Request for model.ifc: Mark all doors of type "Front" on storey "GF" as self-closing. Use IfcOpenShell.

First a look at what the model holds.

```python
import ifcopenshell
import ifcopenshell.util.element

model = ifcopenshell.open("model.ifc")
print(model.schema)
storey = next(s for s in model.by_type("IfcBuildingStorey") if s.Name == "GF")
doors = [e for e in ifcopenshell.util.element.get_decomposition(storey) if e.is_a("IfcDoor")]
seen = {}
for e in doors:
    element_type = ifcopenshell.util.element.get_type(e)
    key = (element_type.Name if element_type != e and element_type else None, ifcopenshell.util.element.get_pset(e, "Pset_DoorCommon", "SelfClosing"))
    seen[key] = seen.get(key, 0) + 1
for (name, value), count in sorted(seen.items(), key=str):
    print(count, "x", name, "|", value)
```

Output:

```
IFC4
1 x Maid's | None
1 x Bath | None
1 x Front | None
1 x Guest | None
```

```python
import ifcopenshell
import ifcopenshell.api.pset
import ifcopenshell.util.element

model = ifcopenshell.open("model.ifc")

storey = next(s for s in model.by_type("IfcBuildingStorey") if s.Name == "GF")
doors = [e for e in ifcopenshell.util.element.get_decomposition(storey) if e.is_a("IfcDoor")]

count = 0
for e in doors:
    element_type = ifcopenshell.util.element.get_type(e)
    if element_type in (None, e) or element_type.Name != "Front":
        continue
    # add_pset returns the element's existing set when there is one.
    pset = ifcopenshell.api.pset.add_pset(model, product=e, name="Pset_DoorCommon")
    ifcopenshell.api.pset.edit_pset(model, pset=pset, properties={"SelfClosing": True})
    count += 1

print(count, "doors updated")

model.write("model_updated.ifc")
```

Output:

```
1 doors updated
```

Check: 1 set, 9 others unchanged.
